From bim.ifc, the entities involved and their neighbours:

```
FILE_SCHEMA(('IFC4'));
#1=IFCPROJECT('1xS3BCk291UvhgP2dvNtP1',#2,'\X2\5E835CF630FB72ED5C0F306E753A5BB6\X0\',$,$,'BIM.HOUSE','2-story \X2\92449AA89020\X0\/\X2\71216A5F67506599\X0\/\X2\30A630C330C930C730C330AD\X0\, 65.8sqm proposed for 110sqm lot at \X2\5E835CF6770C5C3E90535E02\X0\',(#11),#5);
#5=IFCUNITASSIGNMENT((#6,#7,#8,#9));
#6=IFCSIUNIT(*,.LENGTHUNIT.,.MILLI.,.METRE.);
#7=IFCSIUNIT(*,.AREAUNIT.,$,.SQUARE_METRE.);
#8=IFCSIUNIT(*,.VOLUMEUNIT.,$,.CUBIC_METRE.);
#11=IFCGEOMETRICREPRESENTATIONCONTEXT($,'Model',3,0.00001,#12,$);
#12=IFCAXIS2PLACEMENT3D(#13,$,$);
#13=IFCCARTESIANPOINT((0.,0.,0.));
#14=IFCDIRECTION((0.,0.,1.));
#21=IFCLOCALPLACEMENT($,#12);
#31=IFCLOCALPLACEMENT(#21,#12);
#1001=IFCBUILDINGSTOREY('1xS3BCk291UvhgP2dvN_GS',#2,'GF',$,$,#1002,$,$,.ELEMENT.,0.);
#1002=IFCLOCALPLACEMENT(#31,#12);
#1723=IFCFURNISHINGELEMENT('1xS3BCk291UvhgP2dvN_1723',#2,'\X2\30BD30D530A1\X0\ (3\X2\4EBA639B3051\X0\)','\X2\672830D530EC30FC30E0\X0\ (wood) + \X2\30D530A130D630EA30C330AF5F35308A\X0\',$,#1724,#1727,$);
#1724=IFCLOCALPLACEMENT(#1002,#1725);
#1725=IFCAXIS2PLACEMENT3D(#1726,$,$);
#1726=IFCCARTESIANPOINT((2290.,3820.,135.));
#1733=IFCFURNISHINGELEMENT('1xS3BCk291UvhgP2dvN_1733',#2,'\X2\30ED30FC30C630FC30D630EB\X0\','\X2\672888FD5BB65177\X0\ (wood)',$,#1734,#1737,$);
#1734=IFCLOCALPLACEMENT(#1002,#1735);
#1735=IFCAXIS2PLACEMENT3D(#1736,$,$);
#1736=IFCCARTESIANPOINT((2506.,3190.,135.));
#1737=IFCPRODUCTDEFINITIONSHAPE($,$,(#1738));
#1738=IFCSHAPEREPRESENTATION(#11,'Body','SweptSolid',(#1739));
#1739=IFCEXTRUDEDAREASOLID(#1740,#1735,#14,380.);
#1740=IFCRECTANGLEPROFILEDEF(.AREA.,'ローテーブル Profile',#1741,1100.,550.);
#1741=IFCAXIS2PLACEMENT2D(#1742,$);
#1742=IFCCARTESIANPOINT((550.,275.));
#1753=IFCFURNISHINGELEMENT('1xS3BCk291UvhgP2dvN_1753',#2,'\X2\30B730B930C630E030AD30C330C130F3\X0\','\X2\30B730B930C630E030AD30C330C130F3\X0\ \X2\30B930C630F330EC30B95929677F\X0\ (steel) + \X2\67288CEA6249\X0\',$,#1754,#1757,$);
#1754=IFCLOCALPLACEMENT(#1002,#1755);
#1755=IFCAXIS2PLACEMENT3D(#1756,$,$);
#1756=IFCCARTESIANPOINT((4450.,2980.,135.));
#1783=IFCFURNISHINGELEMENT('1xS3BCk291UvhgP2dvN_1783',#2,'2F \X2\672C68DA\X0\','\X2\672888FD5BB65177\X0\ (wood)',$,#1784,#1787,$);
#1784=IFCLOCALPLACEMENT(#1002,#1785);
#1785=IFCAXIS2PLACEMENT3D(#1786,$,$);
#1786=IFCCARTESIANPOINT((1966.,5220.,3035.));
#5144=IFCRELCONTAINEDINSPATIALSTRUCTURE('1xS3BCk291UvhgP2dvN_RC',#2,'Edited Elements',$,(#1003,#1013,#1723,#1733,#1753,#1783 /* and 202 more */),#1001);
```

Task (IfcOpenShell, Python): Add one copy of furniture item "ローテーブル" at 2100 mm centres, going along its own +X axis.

```python
import ifcopenshell
import ifcopenshell.api.geometry
import ifcopenshell.api.root
import ifcopenshell.util.element
import ifcopenshell.util.placement

model = ifcopenshell.open("bim.ifc")


def reuse_history(source, copy):
    """copy_class also copies each property set's owner history, people and application; keep the originals."""
    for rel in copy.IsDefinedBy:
        if rel.is_a("IfcRelDefinesByProperties") and (history := rel.RelatingPropertyDefinition.OwnerHistory):
            rel.RelatingPropertyDefinition.OwnerHistory = source.OwnerHistory
            ifcopenshell.util.element.remove_deep2(model, history)


source = model.by_guid("1xS3BCk291UvhgP2dvN_1733")
base = ifcopenshell.util.placement.get_local_placement(source.ObjectPlacement)
step = base[:3, 0] * 2100.0

for i in range(1, 2):
    copy = ifcopenshell.api.root.copy_class(model, product=source)
    copy.Representation = ifcopenshell.util.element.copy_deep(
        model, source.Representation, exclude=["IfcGeometricRepresentationContext", "IfcRepresentationMap"]
    )
    reuse_history(source, copy)
    matrix = base.copy()
    matrix[:3, 3] += i * step
    print("added at", matrix[:3, 3].round(3) + 0.0)
    ifcopenshell.api.geometry.edit_object_placement(model, product=copy, matrix=matrix, is_si=False)

model.write("bim_edited.ifc")
```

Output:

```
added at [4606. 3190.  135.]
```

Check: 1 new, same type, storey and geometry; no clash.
